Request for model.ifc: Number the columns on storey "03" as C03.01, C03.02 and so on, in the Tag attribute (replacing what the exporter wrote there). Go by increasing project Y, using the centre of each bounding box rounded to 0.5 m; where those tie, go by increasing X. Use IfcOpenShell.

First a look at what the model holds.

```python
import ifcopenshell
import ifcopenshell.util.element
import ifcopenshell.util.placement

model = ifcopenshell.open("model.ifc")
print(model.schema)
storey = next(s for s in model.by_type("IfcBuildingStorey") if s.Name == "03")
columns = [e for e in ifcopenshell.util.element.get_decomposition(storey) if e.is_a("IfcColumn")]
for e in sorted(columns, key=lambda e: e.id()):
    origin = ifcopenshell.util.placement.get_local_placement(e.ObjectPlacement)[:3, 3]
    print(e.id(), e.Tag, e.Name, origin.round(2) + 0.0, sep=" | ")
```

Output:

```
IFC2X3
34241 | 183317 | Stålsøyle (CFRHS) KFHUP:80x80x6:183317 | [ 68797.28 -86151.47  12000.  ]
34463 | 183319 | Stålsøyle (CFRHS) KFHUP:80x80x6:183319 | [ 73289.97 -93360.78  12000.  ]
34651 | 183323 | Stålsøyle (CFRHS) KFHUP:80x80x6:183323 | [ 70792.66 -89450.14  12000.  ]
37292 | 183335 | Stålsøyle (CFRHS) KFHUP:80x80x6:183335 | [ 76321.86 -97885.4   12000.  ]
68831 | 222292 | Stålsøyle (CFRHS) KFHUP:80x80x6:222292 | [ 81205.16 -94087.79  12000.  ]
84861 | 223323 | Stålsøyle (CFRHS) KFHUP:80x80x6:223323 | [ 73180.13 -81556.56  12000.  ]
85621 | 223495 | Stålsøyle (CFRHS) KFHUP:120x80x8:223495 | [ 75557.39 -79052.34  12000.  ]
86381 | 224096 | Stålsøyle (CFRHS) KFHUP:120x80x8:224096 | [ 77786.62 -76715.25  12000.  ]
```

```python
import ifcopenshell
import ifcopenshell.geom
import ifcopenshell.util.element
import ifcopenshell.util.shape

model = ifcopenshell.open("model.ifc")
settings = ifcopenshell.geom.settings()
settings.set("use-world-coords", True)


def centre(element):
    shape = ifcopenshell.geom.create_shape(settings, element)
    return ifcopenshell.util.shape.get_bbox_centroid(shape.geometry)


storey = next(s for s in model.by_type("IfcBuildingStorey") if s.Name == "03")
columns = [e for e in ifcopenshell.util.element.get_decomposition(storey) if e.is_a("IfcColumn")]

# Insertion points can sit at a corner or the storey origin, so sort by the geometry (in metres).
centres = {e: centre(e) for e in columns}
columns.sort(key=lambda e: (round(centres[e][1] / 0.5), centres[e][0]))

for i, e in enumerate(columns, start=1):
    number = f"C03.{i:02d}"
    e.Tag = number
    print(e.id(), number)

model.write("model_edited.ifc")
```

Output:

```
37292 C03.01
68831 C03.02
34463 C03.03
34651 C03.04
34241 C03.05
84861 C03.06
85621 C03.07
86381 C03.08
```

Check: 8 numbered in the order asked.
